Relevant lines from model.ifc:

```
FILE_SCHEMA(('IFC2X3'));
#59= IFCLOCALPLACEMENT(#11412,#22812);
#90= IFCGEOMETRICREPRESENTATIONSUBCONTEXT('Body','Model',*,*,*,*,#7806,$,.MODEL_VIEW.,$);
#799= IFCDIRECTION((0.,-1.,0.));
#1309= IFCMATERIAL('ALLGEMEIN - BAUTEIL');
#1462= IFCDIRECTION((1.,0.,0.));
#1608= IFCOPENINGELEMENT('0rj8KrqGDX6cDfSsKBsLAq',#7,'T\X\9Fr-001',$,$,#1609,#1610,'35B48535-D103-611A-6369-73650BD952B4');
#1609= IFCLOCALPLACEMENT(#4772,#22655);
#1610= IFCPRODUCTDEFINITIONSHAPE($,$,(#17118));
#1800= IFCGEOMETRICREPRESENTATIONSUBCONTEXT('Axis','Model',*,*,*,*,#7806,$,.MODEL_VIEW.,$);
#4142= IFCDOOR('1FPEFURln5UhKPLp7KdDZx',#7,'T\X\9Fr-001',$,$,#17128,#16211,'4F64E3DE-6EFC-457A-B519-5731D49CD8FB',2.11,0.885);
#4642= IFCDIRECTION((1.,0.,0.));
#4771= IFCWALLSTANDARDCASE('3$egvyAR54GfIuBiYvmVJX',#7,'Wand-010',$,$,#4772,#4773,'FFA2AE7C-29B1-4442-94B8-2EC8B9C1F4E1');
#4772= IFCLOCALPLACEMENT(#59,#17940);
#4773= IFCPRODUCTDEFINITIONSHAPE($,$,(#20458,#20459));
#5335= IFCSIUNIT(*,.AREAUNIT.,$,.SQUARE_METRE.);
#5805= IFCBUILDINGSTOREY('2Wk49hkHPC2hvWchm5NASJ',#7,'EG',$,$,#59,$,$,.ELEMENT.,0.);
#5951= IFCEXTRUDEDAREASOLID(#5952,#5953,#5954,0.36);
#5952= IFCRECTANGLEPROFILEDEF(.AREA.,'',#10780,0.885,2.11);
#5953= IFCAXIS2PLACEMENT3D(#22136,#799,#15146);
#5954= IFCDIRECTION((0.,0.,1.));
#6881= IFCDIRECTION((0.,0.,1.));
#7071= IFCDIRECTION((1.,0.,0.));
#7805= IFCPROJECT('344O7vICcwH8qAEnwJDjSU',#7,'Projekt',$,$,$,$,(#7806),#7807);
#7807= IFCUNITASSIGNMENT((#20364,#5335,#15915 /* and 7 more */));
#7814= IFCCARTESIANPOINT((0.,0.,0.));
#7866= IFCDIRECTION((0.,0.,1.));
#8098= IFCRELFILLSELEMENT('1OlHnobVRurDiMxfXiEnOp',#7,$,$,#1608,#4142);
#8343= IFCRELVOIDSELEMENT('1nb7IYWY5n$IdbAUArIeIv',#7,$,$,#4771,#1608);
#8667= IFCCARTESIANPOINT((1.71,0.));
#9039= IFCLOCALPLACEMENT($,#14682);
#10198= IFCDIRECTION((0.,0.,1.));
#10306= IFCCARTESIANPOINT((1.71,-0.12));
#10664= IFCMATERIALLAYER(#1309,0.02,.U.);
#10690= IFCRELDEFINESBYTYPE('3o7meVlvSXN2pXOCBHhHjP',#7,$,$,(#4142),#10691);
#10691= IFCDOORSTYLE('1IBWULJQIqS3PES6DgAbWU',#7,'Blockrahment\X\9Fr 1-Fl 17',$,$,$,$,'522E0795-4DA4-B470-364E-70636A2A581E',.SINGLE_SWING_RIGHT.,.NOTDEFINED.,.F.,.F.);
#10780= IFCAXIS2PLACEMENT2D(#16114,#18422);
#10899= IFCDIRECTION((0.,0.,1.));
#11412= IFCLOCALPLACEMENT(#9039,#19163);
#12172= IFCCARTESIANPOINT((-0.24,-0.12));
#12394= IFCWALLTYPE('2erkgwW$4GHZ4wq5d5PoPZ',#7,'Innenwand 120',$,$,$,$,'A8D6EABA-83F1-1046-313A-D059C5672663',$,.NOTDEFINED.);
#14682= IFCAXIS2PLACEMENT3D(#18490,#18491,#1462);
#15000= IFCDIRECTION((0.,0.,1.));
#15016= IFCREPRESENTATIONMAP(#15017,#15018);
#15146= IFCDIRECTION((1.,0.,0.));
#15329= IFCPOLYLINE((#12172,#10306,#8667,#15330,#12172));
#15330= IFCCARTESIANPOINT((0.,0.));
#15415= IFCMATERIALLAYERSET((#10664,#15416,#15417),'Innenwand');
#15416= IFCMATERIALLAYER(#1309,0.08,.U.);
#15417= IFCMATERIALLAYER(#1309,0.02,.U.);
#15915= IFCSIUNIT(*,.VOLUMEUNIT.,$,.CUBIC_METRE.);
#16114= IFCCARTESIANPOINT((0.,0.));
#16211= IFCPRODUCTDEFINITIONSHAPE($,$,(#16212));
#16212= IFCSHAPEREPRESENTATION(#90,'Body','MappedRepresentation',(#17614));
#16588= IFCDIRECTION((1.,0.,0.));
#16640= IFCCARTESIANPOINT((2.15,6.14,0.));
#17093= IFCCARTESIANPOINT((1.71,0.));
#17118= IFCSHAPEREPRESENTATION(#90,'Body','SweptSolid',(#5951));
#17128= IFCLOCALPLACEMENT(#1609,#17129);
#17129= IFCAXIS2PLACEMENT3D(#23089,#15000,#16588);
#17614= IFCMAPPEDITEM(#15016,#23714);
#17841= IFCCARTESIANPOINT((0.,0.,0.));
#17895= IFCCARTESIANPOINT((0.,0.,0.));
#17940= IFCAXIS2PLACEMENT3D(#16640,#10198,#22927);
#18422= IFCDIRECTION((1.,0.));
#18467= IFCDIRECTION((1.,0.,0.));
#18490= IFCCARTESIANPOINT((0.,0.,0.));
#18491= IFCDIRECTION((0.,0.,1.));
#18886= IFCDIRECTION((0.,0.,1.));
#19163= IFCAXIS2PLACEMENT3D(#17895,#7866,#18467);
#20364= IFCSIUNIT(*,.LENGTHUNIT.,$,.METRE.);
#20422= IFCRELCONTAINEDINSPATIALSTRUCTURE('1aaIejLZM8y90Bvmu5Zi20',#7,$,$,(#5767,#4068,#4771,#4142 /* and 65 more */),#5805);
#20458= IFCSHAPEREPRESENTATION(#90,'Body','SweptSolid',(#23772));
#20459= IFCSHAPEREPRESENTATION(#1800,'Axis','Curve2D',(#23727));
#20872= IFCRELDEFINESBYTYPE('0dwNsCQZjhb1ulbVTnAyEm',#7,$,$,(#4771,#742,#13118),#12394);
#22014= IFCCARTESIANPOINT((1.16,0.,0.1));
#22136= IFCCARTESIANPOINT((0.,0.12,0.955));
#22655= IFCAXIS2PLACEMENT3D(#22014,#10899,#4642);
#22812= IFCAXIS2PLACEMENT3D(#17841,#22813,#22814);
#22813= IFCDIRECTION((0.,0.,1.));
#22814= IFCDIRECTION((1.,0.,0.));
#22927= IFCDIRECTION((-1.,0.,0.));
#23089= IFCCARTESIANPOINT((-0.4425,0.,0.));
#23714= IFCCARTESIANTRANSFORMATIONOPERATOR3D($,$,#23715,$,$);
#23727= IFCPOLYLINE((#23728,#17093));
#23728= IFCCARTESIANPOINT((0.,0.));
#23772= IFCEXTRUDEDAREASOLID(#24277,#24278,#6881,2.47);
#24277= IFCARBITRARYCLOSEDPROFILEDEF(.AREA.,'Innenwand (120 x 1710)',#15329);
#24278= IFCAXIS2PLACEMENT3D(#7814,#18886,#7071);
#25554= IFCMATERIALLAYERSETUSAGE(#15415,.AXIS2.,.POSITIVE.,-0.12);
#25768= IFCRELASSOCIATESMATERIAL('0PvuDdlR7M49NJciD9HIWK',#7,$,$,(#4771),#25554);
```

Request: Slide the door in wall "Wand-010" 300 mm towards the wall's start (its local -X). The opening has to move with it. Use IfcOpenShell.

```python
import ifcopenshell
import ifcopenshell.api.geometry
import ifcopenshell.util.placement
import ifcopenshell.util.unit

model = ifcopenshell.open("model.ifc")
unit_scale = ifcopenshell.util.unit.calculate_unit_scale(model)

door = model.by_guid("1FPEFURln5UhKPLp7KdDZx")
opening = door.FillsVoids[0].RelatingOpeningElement
wall = opening.VoidsElements[0].RelatingBuildingElement

wall_matrix = ifcopenshell.util.placement.get_local_placement(wall.ObjectPlacement)
shift = wall_matrix[:3, 0] * -0.3 / unit_scale
before = ifcopenshell.util.placement.get_local_placement(door.ObjectPlacement)[:3, 3].copy()

# The door is placed relative to its opening, so it follows when the opening moves.
matrix = ifcopenshell.util.placement.get_local_placement(opening.ObjectPlacement)
matrix[:3, 3] += shift
ifcopenshell.api.geometry.edit_object_placement(
    model, product=opening, matrix=matrix, is_si=False, should_transform_children=True
)

after = ifcopenshell.util.placement.get_local_placement(door.ObjectPlacement)[:3, 3]
print("door moved by", (after - before).round(3) + 0.0)

model.write("model-out.ifc")
```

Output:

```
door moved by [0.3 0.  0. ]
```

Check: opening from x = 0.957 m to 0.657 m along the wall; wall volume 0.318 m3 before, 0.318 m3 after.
